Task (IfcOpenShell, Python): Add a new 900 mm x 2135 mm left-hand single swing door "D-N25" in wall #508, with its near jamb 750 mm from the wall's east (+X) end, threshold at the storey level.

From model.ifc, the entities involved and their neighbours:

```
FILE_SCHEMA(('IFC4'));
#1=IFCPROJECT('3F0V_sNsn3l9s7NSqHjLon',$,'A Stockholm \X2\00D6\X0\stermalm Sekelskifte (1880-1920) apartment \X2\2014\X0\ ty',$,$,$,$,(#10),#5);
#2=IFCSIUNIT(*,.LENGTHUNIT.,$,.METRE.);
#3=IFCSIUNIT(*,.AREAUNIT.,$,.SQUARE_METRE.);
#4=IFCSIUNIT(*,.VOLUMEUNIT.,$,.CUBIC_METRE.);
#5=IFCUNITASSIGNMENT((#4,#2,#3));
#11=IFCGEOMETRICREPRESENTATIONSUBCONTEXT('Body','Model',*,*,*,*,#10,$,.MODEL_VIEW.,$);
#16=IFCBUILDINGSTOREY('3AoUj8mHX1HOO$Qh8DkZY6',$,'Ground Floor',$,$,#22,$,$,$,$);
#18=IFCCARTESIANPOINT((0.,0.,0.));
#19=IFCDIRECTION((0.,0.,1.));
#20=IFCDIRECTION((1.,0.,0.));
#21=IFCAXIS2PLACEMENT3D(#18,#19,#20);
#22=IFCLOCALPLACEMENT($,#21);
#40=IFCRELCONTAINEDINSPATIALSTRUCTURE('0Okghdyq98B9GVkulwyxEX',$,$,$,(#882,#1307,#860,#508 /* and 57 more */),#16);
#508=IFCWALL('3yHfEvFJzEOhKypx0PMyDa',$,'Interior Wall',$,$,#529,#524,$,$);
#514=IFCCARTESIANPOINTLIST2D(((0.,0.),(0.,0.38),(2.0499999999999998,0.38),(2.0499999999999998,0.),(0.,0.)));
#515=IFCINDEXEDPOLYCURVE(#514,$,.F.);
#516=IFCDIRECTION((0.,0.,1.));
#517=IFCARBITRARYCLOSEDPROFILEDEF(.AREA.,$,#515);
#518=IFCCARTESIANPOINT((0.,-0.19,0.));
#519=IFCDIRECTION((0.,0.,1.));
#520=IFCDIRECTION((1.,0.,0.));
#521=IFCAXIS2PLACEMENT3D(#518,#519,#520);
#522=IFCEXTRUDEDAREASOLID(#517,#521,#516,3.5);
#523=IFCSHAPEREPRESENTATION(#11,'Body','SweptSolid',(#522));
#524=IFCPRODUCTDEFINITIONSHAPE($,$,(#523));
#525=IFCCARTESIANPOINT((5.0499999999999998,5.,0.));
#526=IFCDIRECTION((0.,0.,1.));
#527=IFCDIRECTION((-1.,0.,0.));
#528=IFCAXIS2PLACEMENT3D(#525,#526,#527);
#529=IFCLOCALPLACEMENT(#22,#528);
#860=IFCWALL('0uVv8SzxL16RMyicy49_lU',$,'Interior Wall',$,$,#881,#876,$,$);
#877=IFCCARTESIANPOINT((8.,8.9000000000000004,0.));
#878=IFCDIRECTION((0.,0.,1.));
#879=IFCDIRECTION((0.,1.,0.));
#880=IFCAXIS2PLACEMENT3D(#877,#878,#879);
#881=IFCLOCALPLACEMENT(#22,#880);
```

```python
import numpy as np
import ifcopenshell
import ifcopenshell.api.feature
import ifcopenshell.api.geometry
import ifcopenshell.api.root
import ifcopenshell.api.spatial
import ifcopenshell.geom
import ifcopenshell.util.element
import ifcopenshell.util.placement
import ifcopenshell.util.representation
import ifcopenshell.util.shape
import ifcopenshell.util.unit

model = ifcopenshell.open("model.ifc")
unit_scale = ifcopenshell.util.unit.calculate_unit_scale(model)
settings = ifcopenshell.geom.settings()


def volume(element):
    """Net volume in cubic metres, openings subtracted."""
    shape = ifcopenshell.geom.create_shape(settings, element)
    return ifcopenshell.util.shape.get_volume(shape.geometry)


wall = model.by_id(508)
storey = ifcopenshell.util.element.get_container(wall, ifc_class="IfcBuildingStorey")
context = ifcopenshell.util.representation.get_context(model, "Model", "Body", "MODEL_VIEW")
before = volume(wall)

width, height, from_end, sill = 0.9, 2.135, 0.75, 0.0  # metres

# The wall runs along its own X axis, and the end named is its -X end.
wall_shape = ifcopenshell.geom.create_shape(settings, wall)
x, y, z = ifcopenshell.util.shape.get_vertices(wall_shape.geometry).T
start = x.min() + from_end
face, thickness = float(y.min()), float(y.max() - y.min())
wall_matrix = ifcopenshell.util.placement.get_local_placement(wall.ObjectPlacement)
level = ifcopenshell.util.placement.get_local_placement(storey.ObjectPlacement)[2, 3]


def in_wall(x, y):
    """Placement at x, y metres in the wall's axes, at sill height."""
    matrix = wall_matrix.copy()
    matrix[:, 3] = wall_matrix @ np.array([x / unit_scale, y / unit_scale, 0.0, 1.0])
    matrix[2, 3] = level + sill / unit_scale
    return matrix


# Opening: a box that overshoots both wall faces by 50 mm.
opening = ifcopenshell.api.root.create_entity(model, ifc_class="IfcOpeningElement", predefined_type="OPENING")
box = ifcopenshell.api.geometry.add_wall_representation(
    model, context=context, length=width, height=height, thickness=thickness + 0.1
)
ifcopenshell.api.geometry.assign_representation(model, product=opening, representation=box)
ifcopenshell.api.geometry.edit_object_placement(model, product=opening, matrix=in_wall(start, face - 0.05), is_si=False)
ifcopenshell.api.feature.add_feature(model, feature=opening, element=wall)

door = ifcopenshell.api.root.create_entity(model, ifc_class="IfcDoor", name="D-N25", predefined_type="DOOR")
door.OverallWidth, door.OverallHeight = width / unit_scale, height / unit_scale
door.OperationType = "SINGLE_SWING_LEFT"
body = ifcopenshell.api.geometry.add_door_representation(
    model,
    context=context,
    overall_width=door.OverallWidth,
    overall_height=door.OverallHeight,
    operation_type="SINGLE_SWING_LEFT",
    lining_properties={"LiningDepth": thickness / unit_scale, "ThresholdDepth": thickness / unit_scale},
)
ifcopenshell.api.geometry.assign_representation(model, product=door, representation=body)
ifcopenshell.api.spatial.assign_container(model, products=[door], relating_structure=storey)
ifcopenshell.api.feature.add_filling(model, opening=opening, element=door)

# The lining spans the wall, so the door starts at the wall face.
ifcopenshell.api.geometry.edit_object_placement(model, product=door, matrix=in_wall(start, face), is_si=False)

after = volume(wall)

print(f"wall volume {before:.3f} -> {after:.3f} m3")

model.write("model-out.ifc")
```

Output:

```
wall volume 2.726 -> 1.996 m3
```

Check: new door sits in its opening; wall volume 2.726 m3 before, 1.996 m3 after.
